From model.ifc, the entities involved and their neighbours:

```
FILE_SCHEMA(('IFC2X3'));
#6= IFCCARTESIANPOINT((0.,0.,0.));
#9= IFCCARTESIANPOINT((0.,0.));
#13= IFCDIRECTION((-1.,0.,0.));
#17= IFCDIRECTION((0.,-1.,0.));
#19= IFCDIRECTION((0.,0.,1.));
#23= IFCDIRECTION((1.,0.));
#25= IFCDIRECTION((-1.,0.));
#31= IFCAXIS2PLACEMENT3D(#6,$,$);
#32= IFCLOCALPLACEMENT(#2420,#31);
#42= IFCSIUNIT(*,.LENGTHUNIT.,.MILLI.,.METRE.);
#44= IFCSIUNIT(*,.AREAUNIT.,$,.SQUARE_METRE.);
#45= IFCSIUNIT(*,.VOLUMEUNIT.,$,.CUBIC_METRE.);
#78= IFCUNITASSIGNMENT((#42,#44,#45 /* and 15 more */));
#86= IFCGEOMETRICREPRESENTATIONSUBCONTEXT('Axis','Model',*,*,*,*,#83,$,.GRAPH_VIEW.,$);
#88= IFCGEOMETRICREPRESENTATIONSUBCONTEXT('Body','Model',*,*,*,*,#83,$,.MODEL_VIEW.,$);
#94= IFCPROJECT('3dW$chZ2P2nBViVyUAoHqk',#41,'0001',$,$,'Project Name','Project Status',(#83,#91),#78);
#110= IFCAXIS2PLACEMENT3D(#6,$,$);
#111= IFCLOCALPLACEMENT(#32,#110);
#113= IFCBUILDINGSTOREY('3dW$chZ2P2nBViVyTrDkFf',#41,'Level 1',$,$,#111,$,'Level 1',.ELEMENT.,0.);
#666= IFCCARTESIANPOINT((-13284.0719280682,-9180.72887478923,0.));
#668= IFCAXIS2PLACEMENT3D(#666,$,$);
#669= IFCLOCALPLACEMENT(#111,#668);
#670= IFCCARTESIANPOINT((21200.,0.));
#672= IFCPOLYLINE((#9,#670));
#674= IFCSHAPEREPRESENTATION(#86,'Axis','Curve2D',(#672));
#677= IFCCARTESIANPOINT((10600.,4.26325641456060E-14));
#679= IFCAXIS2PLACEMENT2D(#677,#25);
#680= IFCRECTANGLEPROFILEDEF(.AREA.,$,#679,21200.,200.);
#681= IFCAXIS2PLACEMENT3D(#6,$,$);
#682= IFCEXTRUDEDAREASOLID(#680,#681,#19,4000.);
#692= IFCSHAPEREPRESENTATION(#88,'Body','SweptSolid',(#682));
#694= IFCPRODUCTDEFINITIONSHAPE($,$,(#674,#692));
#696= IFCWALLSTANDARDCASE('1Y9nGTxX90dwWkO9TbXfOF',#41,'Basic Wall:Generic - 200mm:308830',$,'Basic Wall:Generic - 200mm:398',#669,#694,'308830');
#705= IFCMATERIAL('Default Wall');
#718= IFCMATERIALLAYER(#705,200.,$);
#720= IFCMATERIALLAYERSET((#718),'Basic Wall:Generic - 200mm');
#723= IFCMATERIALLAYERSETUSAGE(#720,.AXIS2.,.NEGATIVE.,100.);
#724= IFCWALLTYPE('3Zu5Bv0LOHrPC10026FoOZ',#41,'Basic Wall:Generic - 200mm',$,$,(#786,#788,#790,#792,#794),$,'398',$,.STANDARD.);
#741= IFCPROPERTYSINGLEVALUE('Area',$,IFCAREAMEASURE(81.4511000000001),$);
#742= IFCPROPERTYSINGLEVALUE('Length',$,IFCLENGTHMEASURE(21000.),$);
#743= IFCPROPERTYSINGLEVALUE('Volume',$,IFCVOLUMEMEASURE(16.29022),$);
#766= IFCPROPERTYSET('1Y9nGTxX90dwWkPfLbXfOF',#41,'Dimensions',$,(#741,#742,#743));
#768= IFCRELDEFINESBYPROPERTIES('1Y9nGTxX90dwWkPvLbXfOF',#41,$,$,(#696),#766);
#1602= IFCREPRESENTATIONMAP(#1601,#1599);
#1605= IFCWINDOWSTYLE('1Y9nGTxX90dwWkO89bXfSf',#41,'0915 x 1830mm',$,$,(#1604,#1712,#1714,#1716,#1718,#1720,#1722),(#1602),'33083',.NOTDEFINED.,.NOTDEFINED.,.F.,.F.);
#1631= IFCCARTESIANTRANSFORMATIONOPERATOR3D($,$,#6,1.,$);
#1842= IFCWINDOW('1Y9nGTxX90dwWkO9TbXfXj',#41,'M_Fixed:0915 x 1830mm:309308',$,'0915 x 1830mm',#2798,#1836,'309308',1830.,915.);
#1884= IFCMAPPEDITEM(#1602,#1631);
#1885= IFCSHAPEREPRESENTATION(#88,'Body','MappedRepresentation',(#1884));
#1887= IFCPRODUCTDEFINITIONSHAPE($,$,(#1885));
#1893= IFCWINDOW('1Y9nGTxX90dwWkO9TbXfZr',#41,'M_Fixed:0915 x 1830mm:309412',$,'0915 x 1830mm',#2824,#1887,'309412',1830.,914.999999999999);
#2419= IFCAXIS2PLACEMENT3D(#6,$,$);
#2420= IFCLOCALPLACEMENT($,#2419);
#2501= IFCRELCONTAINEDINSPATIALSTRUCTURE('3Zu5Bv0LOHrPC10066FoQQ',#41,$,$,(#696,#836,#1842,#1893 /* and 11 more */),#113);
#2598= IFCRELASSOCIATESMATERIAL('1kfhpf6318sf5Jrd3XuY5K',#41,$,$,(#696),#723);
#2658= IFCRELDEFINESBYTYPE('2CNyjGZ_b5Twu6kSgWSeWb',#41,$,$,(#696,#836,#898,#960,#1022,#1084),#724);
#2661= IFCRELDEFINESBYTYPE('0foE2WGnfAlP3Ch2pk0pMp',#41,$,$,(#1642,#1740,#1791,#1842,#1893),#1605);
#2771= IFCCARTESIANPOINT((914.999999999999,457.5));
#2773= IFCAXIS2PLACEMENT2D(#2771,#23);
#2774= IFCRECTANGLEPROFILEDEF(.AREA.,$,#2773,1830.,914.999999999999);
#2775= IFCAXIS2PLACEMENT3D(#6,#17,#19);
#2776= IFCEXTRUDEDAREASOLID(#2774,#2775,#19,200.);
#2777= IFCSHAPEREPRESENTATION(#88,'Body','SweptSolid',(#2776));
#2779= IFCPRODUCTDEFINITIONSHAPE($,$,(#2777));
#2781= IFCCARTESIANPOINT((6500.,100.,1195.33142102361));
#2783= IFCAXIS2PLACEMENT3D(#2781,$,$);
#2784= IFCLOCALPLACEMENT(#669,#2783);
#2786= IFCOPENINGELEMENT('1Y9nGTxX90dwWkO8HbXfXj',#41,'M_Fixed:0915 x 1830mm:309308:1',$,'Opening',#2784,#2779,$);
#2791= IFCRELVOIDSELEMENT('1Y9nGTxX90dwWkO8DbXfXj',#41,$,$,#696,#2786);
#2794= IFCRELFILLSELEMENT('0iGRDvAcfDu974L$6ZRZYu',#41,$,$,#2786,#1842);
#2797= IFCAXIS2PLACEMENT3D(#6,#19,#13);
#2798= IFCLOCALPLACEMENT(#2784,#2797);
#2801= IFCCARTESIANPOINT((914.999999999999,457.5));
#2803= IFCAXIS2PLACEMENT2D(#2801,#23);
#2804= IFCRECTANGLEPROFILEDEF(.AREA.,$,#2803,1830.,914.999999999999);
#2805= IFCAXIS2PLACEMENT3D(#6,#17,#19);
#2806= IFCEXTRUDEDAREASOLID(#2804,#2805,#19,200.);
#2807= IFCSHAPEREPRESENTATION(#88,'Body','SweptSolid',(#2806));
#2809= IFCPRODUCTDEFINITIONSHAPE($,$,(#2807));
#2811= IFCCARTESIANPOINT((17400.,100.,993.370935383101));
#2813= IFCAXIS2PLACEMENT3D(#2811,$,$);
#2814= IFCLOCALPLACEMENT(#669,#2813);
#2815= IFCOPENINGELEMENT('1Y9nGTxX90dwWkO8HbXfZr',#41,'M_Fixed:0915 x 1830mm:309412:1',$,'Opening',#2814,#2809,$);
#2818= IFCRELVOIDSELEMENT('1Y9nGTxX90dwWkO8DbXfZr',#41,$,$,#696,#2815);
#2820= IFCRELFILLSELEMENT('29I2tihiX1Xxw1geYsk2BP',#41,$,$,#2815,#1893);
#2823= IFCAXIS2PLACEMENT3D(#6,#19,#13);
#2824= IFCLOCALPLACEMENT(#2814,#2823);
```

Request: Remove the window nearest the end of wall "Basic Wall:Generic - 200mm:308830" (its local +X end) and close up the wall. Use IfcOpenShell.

```python
import ifcopenshell
import ifcopenshell.api.feature
import ifcopenshell.api.pset
import ifcopenshell.api.root
import ifcopenshell.geom
import ifcopenshell.util.element
import ifcopenshell.util.shape
import ifcopenshell.util.unit

model = ifcopenshell.open("model.ifc")
area_scale = ifcopenshell.util.unit.calculate_unit_scale(model, "AREAUNIT")
volume_scale = ifcopenshell.util.unit.calculate_unit_scale(model, "VOLUMEUNIT")
settings = ifcopenshell.geom.settings()


def volume(element):
    """Net volume in cubic metres, openings subtracted."""
    shape = ifcopenshell.geom.create_shape(settings, element)
    return ifcopenshell.util.shape.get_volume(shape.geometry)


window = model.by_id(1893)
opening = window.FillsVoids[0].RelatingOpeningElement
wall = opening.VoidsElements[0].RelatingBuildingElement
before = volume(wall)

ifcopenshell.api.root.remove_product(model, product=window)
ifcopenshell.api.feature.remove_feature(model, feature=opening)

after = volume(wall)
thickness = 0.2  # wall thickness in metres

# Update the wall's stored quantities.
pset = model.by_id(ifcopenshell.util.element.get_pset(wall, "Dimensions", should_inherit=False)["id"])
ifcopenshell.api.pset.edit_pset(model, pset=pset, properties={
    "Area": model.create_entity("IfcAreaMeasure", after / thickness / area_scale),
    "Volume": model.create_entity("IfcVolumeMeasure", after / volume_scale),
})

print(f"wall volume {before:.3f} -> {after:.3f} m3")

model.write("model_rev.ifc")
```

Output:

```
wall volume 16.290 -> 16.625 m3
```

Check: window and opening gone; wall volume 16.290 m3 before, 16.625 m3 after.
